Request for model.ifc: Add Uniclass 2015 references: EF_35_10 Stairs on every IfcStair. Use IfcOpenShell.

First a look at what the model holds.

```python
import ifcopenshell

model = ifcopenshell.open("model.ifc")
print(model.schema)
print("classifications:", [c.Name for c in model.by_type("IfcClassification")])
for ifc_class in ("IfcDoor", "IfcRoof", "IfcStair", "IfcWall", "IfcWindow"):
    print(ifc_class, len(model.by_type(ifc_class)))
```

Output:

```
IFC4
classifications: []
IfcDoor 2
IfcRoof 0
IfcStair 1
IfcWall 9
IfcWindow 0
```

```python
import ifcopenshell
import ifcopenshell.api.classification

model = ifcopenshell.open("model.ifc")

system = ifcopenshell.api.classification.add_classification(model, classification="Uniclass 2015")

codes = {
    "IfcStair": ("EF_35_10", "Stairs"),
}
for ifc_class, (code, name) in codes.items():
    products = model.by_type(ifc_class)
    ifcopenshell.api.classification.add_reference(
        model, products=products, classification=system, identification=code, name=name
    )
    print(code, len(products))

model.write("model_v2.ifc")
```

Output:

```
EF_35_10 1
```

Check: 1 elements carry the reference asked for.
